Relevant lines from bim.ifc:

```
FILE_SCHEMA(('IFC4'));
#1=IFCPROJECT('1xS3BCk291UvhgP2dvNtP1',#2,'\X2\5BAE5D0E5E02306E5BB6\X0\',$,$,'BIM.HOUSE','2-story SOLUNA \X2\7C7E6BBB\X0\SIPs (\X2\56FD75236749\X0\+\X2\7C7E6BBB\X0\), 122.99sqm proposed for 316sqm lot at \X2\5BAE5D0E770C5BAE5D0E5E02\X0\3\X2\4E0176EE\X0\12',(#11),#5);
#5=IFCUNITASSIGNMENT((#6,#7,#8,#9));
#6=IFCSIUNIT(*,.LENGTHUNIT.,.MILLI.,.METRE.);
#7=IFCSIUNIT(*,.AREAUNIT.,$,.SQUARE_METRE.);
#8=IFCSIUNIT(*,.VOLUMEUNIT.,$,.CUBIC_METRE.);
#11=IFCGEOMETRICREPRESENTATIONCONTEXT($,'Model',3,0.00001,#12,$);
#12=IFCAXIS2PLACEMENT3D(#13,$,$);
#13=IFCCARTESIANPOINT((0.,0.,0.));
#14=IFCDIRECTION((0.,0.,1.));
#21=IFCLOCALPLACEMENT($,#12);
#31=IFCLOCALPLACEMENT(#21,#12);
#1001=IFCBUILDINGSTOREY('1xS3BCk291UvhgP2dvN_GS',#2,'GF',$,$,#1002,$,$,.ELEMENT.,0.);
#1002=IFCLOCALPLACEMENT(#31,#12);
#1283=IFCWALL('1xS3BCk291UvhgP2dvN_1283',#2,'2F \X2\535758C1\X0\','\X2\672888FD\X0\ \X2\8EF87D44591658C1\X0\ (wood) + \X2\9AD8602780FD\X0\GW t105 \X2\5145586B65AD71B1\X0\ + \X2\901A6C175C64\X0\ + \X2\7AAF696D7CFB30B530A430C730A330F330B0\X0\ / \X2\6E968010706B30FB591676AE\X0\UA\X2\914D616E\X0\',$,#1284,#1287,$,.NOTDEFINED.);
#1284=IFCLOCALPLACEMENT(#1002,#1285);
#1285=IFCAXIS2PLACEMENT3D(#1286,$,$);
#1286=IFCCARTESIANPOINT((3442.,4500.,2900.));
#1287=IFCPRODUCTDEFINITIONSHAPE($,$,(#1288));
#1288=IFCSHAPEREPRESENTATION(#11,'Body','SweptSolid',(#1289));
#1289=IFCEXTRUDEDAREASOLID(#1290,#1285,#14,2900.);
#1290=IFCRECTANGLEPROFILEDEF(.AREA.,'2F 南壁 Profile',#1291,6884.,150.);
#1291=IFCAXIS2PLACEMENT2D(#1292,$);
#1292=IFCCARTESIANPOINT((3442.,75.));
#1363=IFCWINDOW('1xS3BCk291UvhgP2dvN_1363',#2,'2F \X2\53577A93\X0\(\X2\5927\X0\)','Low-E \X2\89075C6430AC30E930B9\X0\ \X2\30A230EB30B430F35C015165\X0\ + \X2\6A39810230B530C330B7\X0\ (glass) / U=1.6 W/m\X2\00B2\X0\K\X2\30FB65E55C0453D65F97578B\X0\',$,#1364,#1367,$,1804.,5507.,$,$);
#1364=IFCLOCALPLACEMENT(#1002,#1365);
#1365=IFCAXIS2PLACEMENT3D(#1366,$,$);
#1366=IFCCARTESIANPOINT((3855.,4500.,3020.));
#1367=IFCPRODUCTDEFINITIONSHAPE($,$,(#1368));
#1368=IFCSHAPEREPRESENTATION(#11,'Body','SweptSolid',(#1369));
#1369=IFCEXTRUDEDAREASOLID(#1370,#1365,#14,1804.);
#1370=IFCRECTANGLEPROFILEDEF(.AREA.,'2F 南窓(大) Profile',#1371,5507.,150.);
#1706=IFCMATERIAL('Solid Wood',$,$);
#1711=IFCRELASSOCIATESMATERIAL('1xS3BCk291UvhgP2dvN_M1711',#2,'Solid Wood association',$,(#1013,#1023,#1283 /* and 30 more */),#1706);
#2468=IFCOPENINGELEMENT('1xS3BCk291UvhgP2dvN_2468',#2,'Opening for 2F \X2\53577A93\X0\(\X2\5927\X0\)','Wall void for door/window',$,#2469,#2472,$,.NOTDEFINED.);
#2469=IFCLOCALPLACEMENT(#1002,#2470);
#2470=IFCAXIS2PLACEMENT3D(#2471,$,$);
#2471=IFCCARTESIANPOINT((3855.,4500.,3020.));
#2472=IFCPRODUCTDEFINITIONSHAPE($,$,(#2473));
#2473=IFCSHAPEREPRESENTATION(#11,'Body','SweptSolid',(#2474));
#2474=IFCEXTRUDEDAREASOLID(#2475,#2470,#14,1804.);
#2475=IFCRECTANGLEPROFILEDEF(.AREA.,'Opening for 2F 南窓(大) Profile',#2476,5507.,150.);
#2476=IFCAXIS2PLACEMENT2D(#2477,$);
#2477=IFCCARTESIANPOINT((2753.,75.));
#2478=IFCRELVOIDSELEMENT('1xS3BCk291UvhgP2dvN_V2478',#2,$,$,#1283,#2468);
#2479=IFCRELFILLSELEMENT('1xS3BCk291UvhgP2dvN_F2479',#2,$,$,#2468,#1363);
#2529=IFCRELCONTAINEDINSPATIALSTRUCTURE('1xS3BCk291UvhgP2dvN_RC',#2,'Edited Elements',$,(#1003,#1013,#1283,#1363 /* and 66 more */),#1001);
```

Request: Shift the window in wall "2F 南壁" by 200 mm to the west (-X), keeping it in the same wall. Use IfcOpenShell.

```python
import ifcopenshell
import ifcopenshell.api.geometry
import ifcopenshell.util.placement

model = ifcopenshell.open("bim.ifc")

window = model.by_guid("1xS3BCk291UvhgP2dvN_1363")
opening = window.FillsVoids[0].RelatingOpeningElement
wall = opening.VoidsElements[0].RelatingBuildingElement

wall_matrix = ifcopenshell.util.placement.get_local_placement(wall.ObjectPlacement)
shift = wall_matrix[:3, 0] * -200.0
before = ifcopenshell.util.placement.get_local_placement(window.ObjectPlacement)[:3, 3].copy()

# The window is not placed relative to its opening, so move both.
for product in (opening, window):
    matrix = ifcopenshell.util.placement.get_local_placement(product.ObjectPlacement)
    matrix[:3, 3] += shift
    ifcopenshell.api.geometry.edit_object_placement(model, product=product, matrix=matrix, is_si=False)

after = ifcopenshell.util.placement.get_local_placement(window.ObjectPlacement)[:3, 3]
print("window moved by", (after - before).round(3) + 0.0)

model.write("bim_edited.ifc")
```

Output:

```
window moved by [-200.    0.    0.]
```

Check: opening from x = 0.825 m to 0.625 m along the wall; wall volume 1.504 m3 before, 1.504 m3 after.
